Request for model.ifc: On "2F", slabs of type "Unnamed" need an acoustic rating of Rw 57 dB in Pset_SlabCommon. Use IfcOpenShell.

First a look at what the model holds.

```python
import ifcopenshell
import ifcopenshell.util.element

model = ifcopenshell.open("model.ifc")
print(model.schema)
storey = next(s for s in model.by_type("IfcBuildingStorey") if s.Name == "2F")
slabs = [e for e in ifcopenshell.util.element.get_decomposition(storey) if e.is_a("IfcSlab")]
seen = {}
for e in slabs:
    element_type = ifcopenshell.util.element.get_type(e)
    key = (element_type.Name if element_type != e and element_type else None, ifcopenshell.util.element.get_pset(e, "Pset_SlabCommon", "AcousticRating"))
    seen[key] = seen.get(key, 0) + 1
for (name, value), count in sorted(seen.items(), key=str):
    print(count, "x", name, "|", value)
```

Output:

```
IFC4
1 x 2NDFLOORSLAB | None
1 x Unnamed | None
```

```python
import ifcopenshell
import ifcopenshell.api.pset
import ifcopenshell.util.element

model = ifcopenshell.open("model.ifc")

storey = next(s for s in model.by_type("IfcBuildingStorey") if s.Name == "2F")
slabs = [e for e in ifcopenshell.util.element.get_decomposition(storey) if e.is_a("IfcSlab")]

count = 0
for e in slabs:
    element_type = ifcopenshell.util.element.get_type(e)
    if element_type in (None, e) or element_type.Name != "Unnamed":
        continue
    # add_pset returns the element's existing set when there is one.
    pset = ifcopenshell.api.pset.add_pset(model, product=e, name="Pset_SlabCommon")
    ifcopenshell.api.pset.edit_pset(model, pset=pset, properties={"AcousticRating": "Rw 57 dB"})
    count += 1

print(count, "slabs updated")

model.write("model_rev.ifc")
```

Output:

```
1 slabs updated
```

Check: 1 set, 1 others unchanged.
